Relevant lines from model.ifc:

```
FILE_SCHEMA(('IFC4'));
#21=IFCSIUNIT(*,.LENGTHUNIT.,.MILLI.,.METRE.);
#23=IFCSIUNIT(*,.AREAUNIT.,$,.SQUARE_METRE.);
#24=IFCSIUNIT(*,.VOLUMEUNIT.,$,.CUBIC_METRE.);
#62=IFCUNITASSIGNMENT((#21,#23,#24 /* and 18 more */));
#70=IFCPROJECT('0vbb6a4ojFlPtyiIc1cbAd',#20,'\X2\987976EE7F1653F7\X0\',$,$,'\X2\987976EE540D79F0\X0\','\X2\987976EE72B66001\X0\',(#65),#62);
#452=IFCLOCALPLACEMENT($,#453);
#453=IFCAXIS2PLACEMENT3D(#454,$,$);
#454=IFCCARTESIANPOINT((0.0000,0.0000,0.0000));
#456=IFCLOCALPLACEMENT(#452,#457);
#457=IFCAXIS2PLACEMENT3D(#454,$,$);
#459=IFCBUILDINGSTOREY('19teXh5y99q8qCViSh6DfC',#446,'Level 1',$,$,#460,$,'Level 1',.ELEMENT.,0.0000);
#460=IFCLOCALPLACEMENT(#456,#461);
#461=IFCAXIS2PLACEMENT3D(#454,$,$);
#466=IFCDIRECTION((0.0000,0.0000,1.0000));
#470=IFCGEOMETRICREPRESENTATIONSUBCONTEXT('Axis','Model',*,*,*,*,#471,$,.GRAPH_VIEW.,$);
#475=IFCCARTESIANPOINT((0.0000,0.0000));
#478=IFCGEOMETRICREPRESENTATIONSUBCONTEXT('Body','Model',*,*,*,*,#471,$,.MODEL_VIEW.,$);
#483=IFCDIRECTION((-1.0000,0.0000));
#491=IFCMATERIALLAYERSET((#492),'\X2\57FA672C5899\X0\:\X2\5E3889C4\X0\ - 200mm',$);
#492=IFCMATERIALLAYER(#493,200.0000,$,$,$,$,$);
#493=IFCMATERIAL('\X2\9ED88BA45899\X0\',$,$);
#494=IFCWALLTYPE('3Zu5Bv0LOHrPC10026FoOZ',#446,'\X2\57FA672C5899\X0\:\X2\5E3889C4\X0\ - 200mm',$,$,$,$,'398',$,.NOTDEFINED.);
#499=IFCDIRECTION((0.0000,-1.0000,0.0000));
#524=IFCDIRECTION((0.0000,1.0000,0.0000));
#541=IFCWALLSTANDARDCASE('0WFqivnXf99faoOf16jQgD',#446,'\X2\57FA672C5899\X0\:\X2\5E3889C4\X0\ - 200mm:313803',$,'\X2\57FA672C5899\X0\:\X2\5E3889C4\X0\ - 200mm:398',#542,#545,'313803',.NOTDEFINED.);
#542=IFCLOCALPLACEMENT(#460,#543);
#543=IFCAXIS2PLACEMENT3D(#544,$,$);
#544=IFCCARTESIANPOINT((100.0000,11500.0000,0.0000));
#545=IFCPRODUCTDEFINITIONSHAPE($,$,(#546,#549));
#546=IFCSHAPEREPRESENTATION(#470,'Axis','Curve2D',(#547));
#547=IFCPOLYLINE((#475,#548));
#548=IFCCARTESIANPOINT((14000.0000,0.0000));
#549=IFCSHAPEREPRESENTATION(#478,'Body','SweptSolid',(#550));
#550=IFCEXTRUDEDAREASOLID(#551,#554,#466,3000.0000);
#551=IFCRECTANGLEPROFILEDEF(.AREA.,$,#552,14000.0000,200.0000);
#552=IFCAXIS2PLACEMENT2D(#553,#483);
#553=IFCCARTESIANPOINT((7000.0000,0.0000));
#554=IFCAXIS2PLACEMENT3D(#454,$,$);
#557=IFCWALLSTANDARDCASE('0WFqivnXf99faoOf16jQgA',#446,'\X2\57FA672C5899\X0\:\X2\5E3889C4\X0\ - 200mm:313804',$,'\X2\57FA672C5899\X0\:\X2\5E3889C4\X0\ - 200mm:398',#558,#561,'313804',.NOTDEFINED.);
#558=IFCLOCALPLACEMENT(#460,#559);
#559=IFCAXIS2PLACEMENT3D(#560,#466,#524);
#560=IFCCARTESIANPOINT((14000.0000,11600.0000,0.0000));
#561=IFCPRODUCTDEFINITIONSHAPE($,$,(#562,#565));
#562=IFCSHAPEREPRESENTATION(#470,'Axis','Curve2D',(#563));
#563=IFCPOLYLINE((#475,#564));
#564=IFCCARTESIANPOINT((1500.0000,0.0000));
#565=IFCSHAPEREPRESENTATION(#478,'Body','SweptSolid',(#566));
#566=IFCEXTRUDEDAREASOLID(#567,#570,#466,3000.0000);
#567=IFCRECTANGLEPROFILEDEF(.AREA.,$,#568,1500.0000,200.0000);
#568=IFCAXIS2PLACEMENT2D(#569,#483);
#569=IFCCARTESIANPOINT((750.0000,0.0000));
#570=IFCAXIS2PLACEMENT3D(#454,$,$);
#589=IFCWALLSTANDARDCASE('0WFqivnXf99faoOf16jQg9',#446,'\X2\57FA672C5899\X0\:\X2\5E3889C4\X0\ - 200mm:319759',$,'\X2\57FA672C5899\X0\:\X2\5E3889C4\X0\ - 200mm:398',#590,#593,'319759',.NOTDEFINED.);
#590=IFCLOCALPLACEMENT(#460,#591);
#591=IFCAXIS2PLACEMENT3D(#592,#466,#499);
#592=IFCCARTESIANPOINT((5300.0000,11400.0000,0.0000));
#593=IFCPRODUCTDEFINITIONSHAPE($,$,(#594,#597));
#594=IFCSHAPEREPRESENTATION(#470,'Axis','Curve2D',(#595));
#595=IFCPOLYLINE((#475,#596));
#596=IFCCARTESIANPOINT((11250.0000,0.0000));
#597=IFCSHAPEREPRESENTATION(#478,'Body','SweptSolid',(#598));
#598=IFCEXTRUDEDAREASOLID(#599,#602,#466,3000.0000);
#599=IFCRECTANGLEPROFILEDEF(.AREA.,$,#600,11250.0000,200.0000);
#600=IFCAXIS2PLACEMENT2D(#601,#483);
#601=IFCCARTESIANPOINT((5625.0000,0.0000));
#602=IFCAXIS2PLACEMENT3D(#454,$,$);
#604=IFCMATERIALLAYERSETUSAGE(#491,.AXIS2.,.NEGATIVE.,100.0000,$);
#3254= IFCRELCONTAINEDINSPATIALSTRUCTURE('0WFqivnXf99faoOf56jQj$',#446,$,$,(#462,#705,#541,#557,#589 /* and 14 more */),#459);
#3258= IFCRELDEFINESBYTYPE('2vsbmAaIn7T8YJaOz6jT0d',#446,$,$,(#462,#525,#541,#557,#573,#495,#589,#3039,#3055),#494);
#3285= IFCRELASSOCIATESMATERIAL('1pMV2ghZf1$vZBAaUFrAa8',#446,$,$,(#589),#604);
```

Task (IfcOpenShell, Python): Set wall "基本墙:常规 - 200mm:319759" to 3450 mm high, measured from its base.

```python
import ifcopenshell
import ifcopenshell.geom
import ifcopenshell.util.representation
import ifcopenshell.util.shape
import ifcopenshell.util.unit

model = ifcopenshell.open("model.ifc")
unit_scale = ifcopenshell.util.unit.calculate_unit_scale(model)
settings = ifcopenshell.geom.settings()


def volume(element):
    """Net volume in cubic metres, openings subtracted."""
    shape = ifcopenshell.geom.create_shape(settings, element)
    return ifcopenshell.util.shape.get_volume(shape.geometry)


wall = model.by_guid("0WFqivnXf99faoOf16jQg9")
before = volume(wall)

body = ifcopenshell.util.representation.get_representation(wall, "Model", "Body")
solid = body.Items[0]
old_height = solid.Depth
solid.Depth = 3.45 / unit_scale
after = volume(wall)

print(f"height {old_height:g} -> {solid.Depth:g}, volume {before:.3f} -> {after:.3f} m3")

model.write("model_edited.ifc")
```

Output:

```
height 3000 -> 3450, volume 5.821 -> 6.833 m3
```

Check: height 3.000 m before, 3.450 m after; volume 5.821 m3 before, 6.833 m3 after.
